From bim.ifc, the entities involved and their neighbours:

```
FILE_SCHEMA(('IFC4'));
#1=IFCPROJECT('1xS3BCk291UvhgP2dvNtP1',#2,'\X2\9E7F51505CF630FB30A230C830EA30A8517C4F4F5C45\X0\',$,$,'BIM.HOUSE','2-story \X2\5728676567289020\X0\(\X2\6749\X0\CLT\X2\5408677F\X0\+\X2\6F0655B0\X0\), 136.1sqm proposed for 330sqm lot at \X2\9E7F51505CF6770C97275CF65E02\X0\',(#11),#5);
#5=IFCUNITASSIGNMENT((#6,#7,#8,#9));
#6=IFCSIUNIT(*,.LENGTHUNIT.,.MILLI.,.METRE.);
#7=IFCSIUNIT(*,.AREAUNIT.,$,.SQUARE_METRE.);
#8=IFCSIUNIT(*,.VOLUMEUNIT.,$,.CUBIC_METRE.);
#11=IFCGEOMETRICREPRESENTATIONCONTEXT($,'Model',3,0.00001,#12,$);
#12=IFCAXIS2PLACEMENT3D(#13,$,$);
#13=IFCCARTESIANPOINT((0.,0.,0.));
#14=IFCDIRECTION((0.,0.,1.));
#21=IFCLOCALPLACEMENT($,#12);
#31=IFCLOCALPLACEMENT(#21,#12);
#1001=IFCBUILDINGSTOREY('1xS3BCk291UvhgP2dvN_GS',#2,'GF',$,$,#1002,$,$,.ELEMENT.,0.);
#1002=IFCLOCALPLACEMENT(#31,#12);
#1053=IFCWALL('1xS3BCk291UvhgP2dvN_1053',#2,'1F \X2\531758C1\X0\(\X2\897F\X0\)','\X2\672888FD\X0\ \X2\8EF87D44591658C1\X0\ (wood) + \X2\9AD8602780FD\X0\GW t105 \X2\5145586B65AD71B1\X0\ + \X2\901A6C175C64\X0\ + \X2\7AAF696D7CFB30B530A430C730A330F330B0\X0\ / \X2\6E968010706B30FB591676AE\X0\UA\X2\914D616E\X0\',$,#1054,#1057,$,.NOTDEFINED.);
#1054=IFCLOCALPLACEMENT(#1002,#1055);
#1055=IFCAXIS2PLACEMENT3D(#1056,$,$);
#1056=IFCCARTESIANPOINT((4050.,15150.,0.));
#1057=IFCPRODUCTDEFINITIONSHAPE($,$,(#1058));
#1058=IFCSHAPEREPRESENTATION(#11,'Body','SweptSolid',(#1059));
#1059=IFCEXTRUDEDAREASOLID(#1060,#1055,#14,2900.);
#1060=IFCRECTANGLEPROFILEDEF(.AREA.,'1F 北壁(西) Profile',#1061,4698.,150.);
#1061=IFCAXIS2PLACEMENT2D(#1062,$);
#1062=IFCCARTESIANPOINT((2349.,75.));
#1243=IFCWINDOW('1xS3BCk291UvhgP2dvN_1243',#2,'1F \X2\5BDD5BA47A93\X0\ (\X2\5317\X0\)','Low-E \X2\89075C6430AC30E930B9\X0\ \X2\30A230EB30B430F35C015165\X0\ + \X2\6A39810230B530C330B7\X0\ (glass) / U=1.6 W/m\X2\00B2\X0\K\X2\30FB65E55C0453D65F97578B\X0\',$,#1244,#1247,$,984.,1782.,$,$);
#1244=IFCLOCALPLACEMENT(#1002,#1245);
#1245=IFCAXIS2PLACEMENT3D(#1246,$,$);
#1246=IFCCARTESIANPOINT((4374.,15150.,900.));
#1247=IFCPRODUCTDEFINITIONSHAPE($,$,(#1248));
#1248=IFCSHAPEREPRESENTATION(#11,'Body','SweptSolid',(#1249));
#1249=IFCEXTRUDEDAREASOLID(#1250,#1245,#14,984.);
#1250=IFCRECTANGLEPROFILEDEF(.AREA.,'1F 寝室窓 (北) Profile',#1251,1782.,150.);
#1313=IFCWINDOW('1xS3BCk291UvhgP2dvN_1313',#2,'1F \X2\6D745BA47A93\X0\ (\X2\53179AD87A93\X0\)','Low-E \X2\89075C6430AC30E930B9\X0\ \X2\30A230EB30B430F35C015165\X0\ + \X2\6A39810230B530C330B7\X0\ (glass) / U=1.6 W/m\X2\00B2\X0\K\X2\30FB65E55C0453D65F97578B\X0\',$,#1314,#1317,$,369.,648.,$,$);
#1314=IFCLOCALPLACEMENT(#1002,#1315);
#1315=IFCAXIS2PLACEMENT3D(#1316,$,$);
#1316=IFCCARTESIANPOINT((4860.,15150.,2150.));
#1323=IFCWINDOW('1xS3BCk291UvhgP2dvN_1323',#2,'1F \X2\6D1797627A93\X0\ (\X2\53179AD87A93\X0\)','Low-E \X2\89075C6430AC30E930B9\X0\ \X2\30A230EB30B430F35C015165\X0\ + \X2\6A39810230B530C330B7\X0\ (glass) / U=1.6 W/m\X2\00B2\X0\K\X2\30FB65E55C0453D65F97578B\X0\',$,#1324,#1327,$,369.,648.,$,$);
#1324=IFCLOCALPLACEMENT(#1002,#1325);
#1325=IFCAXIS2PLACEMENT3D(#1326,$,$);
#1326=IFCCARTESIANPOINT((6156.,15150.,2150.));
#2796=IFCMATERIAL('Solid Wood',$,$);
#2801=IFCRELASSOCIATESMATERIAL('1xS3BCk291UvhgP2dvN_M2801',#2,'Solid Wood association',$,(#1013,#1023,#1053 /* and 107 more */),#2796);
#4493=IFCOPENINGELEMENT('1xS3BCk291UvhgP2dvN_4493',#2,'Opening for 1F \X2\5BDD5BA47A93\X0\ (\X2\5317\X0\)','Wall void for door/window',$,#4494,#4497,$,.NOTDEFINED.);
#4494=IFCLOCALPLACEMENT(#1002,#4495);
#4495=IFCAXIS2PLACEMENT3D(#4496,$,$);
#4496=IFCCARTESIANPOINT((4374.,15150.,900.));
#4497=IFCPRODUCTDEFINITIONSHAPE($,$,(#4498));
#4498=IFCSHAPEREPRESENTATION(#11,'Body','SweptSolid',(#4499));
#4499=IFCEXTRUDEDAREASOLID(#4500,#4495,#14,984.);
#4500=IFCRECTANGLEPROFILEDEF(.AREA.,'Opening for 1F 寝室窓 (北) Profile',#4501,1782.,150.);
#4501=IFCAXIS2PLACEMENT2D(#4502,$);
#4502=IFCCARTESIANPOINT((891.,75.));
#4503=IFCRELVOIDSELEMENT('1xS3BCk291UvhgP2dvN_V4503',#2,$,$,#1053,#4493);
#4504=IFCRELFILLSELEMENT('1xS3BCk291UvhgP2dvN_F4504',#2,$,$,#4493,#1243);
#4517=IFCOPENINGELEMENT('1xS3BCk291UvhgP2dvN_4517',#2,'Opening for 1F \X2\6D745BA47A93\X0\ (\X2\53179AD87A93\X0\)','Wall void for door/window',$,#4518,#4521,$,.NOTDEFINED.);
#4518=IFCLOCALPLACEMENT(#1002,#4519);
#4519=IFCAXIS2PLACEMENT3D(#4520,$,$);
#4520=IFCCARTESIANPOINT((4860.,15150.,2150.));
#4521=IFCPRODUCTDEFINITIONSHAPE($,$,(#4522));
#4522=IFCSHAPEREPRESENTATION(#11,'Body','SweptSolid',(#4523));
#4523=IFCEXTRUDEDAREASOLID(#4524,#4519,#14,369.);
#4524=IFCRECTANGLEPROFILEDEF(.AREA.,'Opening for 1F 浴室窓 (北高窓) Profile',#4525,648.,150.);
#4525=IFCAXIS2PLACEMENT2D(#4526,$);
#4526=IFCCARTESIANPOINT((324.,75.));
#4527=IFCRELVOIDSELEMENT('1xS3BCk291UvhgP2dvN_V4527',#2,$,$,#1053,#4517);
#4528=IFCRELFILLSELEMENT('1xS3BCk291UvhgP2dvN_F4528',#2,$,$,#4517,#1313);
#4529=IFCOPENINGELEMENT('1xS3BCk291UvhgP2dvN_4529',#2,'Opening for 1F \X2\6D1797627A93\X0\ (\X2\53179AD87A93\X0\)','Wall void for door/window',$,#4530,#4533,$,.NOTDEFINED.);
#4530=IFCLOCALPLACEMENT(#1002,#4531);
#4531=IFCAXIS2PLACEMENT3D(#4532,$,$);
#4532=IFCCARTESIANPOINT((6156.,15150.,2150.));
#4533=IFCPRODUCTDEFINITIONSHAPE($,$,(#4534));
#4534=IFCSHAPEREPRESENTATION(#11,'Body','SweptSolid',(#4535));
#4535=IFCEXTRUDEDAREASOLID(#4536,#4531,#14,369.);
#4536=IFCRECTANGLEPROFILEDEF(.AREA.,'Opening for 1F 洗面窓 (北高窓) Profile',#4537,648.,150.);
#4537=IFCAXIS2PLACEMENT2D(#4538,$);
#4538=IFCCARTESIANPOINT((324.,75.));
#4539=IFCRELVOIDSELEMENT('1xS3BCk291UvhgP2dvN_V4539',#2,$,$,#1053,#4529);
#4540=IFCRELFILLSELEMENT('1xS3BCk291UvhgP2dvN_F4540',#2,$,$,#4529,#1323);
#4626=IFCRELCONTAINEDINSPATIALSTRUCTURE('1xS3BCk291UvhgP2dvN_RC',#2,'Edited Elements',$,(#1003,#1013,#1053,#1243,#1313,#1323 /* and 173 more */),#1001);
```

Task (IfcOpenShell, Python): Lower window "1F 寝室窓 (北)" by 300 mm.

```python
import numpy as np
import ifcopenshell
import ifcopenshell.api.geometry
import ifcopenshell.util.placement
import ifcopenshell.util.unit

model = ifcopenshell.open("bim.ifc")
unit_scale = ifcopenshell.util.unit.calculate_unit_scale(model)

window = model.by_guid("1xS3BCk291UvhgP2dvN_1243")
opening = window.FillsVoids[0].RelatingOpeningElement
dz = -0.3 / unit_scale

shift = np.array([0.0, 0.0, dz])
# The window is not placed relative to its opening, so move both.
for product in (opening, window):
    matrix = ifcopenshell.util.placement.get_local_placement(product.ObjectPlacement)
    matrix[:3, 3] += shift
    ifcopenshell.api.geometry.edit_object_placement(model, product=product, matrix=matrix, is_si=False)

print(f"moved by {dz * unit_scale:+.3f} m")

model.write("bim_edited.ifc")
```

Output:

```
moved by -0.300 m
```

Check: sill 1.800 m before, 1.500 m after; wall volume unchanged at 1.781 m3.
